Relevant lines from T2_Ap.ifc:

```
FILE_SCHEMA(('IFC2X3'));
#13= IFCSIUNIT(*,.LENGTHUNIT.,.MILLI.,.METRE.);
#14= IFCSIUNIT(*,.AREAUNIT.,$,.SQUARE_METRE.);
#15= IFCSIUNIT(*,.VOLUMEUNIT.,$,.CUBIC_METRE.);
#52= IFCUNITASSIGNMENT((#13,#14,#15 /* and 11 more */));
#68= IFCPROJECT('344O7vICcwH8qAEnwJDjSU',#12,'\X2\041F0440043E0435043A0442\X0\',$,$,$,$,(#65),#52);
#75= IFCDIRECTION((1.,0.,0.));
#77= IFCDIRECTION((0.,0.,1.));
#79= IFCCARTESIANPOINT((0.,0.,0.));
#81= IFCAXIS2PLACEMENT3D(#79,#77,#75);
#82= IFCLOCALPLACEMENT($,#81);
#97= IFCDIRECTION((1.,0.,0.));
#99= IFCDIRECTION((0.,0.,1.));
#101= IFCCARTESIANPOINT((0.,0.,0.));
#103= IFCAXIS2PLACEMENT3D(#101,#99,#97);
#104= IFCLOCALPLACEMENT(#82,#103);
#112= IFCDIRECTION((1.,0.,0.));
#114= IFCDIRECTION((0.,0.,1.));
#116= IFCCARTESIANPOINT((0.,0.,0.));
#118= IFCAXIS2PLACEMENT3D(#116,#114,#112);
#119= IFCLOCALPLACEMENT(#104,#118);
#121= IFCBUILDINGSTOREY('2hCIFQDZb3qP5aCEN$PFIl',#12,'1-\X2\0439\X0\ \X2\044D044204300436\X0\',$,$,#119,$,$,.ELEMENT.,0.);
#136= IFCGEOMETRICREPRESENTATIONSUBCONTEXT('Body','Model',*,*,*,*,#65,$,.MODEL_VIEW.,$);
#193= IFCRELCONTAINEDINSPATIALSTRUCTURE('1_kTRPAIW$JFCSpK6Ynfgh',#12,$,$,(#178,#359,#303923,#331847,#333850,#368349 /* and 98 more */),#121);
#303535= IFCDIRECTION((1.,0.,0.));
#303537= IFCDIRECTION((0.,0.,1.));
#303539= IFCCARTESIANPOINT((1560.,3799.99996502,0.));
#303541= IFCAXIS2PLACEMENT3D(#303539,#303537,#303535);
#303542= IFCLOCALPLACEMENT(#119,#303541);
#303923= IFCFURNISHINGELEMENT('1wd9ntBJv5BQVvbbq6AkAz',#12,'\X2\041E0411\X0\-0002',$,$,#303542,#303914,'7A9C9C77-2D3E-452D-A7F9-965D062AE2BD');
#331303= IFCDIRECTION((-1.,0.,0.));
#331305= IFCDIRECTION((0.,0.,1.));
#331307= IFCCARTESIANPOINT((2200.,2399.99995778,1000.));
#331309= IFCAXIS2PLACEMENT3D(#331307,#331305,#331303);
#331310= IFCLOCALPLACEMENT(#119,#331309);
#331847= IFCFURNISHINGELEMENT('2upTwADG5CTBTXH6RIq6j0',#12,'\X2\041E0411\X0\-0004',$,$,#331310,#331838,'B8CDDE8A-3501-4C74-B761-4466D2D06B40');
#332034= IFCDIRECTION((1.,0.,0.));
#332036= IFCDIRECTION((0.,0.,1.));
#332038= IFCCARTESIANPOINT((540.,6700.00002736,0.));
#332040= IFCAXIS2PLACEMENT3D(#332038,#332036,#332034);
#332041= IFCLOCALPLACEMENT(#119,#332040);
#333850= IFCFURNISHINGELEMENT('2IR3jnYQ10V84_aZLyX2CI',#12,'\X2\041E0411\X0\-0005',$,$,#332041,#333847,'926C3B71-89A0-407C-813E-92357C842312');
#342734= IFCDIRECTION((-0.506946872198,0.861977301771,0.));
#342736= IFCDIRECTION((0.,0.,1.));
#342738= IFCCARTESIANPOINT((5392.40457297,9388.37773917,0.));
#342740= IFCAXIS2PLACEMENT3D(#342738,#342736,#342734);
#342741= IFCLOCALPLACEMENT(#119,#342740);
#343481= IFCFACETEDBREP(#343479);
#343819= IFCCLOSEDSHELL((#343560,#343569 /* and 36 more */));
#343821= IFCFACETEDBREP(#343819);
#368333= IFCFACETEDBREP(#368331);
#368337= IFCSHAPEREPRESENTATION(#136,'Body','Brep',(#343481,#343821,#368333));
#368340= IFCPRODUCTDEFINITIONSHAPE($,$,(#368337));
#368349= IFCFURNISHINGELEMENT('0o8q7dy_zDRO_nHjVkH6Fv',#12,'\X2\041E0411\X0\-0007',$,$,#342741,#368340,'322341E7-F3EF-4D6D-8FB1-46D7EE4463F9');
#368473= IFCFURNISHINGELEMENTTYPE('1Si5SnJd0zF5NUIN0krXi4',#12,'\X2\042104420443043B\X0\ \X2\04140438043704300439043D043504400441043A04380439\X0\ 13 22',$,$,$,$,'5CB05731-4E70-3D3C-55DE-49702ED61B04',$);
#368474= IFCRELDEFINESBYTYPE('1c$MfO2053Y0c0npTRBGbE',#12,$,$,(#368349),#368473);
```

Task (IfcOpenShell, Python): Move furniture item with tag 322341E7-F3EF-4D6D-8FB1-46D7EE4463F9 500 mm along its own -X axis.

```python
import ifcopenshell
import ifcopenshell.api.geometry
import ifcopenshell.util.placement

model = ifcopenshell.open("T2_Ap.ifc")

item = model.by_id(368349)
matrix = ifcopenshell.util.placement.get_local_placement(item.ObjectPlacement)
matrix[:3, 3] -= matrix[:3, 0] * 500.0
ifcopenshell.api.geometry.edit_object_placement(model, product=item, matrix=matrix, is_si=False)

print(ifcopenshell.util.placement.get_local_placement(item.ObjectPlacement).round(3) + 0.0)

model.write("T2_Ap_edited.ifc")
```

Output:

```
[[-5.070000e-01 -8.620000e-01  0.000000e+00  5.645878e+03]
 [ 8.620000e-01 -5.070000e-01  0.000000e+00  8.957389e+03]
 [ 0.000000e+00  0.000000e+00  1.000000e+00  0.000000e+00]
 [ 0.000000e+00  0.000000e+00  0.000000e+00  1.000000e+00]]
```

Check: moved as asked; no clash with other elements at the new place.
